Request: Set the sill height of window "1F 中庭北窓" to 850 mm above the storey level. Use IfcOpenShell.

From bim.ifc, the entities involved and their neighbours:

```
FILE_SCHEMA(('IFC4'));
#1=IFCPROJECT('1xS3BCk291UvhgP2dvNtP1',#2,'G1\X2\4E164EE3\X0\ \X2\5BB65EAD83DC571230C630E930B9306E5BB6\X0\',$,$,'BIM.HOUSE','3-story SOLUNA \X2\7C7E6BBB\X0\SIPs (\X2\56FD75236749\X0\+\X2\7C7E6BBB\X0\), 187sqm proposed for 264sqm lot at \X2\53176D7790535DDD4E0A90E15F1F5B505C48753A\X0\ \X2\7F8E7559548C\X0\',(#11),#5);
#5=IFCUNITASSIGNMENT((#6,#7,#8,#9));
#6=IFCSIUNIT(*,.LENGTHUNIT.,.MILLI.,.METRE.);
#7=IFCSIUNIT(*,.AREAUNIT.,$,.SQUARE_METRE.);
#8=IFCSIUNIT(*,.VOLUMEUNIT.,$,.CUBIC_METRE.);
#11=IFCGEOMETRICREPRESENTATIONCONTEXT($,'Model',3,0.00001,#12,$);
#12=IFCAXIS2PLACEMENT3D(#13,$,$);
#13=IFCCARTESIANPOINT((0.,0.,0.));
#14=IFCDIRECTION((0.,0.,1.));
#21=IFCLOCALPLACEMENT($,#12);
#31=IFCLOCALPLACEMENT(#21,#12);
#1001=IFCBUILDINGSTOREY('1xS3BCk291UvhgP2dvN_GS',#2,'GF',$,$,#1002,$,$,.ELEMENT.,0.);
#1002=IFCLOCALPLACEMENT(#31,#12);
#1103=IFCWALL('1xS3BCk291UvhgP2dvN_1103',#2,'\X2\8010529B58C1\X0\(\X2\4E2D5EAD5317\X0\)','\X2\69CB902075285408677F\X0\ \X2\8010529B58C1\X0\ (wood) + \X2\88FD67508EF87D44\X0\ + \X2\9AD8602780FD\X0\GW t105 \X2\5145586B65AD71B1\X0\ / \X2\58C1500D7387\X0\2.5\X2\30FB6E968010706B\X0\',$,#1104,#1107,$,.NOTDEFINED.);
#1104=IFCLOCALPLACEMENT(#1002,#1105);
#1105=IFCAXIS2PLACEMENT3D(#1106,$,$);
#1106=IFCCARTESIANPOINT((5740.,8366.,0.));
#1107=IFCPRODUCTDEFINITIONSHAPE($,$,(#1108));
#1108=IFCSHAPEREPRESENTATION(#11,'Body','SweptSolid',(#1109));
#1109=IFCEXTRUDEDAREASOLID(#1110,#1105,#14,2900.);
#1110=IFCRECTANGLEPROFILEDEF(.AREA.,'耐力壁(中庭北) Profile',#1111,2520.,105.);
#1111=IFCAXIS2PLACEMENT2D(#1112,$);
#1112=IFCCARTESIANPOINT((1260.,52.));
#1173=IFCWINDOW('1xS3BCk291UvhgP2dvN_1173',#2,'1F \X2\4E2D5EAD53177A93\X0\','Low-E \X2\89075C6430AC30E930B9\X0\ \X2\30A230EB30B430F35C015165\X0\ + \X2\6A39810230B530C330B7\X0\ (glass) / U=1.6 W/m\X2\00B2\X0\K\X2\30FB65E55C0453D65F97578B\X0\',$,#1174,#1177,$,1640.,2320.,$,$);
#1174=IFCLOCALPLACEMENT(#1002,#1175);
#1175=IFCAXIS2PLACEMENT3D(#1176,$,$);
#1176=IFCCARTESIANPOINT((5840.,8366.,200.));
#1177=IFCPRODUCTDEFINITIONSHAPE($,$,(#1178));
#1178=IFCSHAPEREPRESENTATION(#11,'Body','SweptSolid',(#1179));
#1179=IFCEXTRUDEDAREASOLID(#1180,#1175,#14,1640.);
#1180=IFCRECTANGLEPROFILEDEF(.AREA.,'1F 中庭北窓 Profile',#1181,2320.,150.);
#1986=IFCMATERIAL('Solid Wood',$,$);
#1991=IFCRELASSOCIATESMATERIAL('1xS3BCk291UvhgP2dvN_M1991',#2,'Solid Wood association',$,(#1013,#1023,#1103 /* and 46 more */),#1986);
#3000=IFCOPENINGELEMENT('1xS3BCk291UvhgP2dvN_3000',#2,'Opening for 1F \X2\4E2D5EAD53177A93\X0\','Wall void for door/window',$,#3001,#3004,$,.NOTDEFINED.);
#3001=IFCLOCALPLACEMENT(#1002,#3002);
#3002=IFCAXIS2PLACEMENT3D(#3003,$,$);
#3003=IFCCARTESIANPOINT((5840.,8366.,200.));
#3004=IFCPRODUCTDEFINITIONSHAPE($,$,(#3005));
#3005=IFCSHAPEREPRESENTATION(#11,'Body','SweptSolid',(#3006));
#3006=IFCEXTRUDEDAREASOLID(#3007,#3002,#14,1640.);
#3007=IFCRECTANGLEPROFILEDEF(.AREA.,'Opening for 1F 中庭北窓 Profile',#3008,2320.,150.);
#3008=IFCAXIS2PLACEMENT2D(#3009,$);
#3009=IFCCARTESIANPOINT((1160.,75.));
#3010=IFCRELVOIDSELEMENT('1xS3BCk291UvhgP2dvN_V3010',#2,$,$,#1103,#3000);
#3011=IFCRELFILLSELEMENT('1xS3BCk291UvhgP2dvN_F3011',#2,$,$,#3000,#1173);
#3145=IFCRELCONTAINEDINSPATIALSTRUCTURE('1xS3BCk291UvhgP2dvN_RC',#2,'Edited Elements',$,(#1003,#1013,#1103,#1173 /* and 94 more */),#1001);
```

```python
import numpy as np
import ifcopenshell
import ifcopenshell.api.geometry
import ifcopenshell.geom
import ifcopenshell.util.element
import ifcopenshell.util.placement
import ifcopenshell.util.shape
import ifcopenshell.util.unit

model = ifcopenshell.open("bim.ifc")
unit_scale = ifcopenshell.util.unit.calculate_unit_scale(model)

window = model.by_guid("1xS3BCk291UvhgP2dvN_1173")
opening = window.FillsVoids[0].RelatingOpeningElement
storey = ifcopenshell.util.element.get_container(window, ifc_class="IfcBuildingStorey")
level = ifcopenshell.util.placement.get_local_placement(storey.ObjectPlacement)[2, 3]

# The opening's origin need not be at the sill, so measure its lowest point.
shape = ifcopenshell.geom.create_shape(ifcopenshell.geom.settings(), opening)
bottom = ifcopenshell.util.shape.get_shape_bottom_elevation(shape, shape.geometry) / unit_scale
dz = level + 850.0 - bottom

shift = np.array([0.0, 0.0, dz])
# The window is not placed relative to its opening, so move both.
for product in (opening, window):
    matrix = ifcopenshell.util.placement.get_local_placement(product.ObjectPlacement)
    matrix[:3, 3] += shift
    ifcopenshell.api.geometry.edit_object_placement(model, product=product, matrix=matrix, is_si=False)

print(f"moved by {dz * unit_scale:+.3f} m")

model.write("bim_v2.ifc")
```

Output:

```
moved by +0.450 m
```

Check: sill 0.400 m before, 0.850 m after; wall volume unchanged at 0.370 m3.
